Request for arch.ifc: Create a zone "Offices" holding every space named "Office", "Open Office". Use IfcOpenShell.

First a look at what the model holds.

```python
import ifcopenshell

model = ifcopenshell.open("arch.ifc")
print(model.schema)
seen = {}
for space in model.by_type("IfcSpace"):
    seen[space.LongName] = seen.get(space.LongName, 0) + 1
for name, count in sorted(seen.items(), key=str):
    print(count, "x", name)
print("zones:", [z.Name for z in model.by_type("IfcZone")][:20])
```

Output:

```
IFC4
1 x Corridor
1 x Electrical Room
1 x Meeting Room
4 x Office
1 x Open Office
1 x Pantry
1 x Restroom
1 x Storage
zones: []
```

```python
import ifcopenshell
import ifcopenshell.api.group
import ifcopenshell.api.root

model = ifcopenshell.open("arch.ifc")

names = {"Office", "Open Office"}
spaces = [s for s in model.by_type("IfcSpace") if s.LongName in names]

zone = ifcopenshell.api.root.create_entity(model, ifc_class="IfcZone", name="Offices")
ifcopenshell.api.group.assign_group(model, products=spaces, group=zone)
print(len(spaces), "spaces in", zone.Name)

model.write("arch_updated.ifc")
```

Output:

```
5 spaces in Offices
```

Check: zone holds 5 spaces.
